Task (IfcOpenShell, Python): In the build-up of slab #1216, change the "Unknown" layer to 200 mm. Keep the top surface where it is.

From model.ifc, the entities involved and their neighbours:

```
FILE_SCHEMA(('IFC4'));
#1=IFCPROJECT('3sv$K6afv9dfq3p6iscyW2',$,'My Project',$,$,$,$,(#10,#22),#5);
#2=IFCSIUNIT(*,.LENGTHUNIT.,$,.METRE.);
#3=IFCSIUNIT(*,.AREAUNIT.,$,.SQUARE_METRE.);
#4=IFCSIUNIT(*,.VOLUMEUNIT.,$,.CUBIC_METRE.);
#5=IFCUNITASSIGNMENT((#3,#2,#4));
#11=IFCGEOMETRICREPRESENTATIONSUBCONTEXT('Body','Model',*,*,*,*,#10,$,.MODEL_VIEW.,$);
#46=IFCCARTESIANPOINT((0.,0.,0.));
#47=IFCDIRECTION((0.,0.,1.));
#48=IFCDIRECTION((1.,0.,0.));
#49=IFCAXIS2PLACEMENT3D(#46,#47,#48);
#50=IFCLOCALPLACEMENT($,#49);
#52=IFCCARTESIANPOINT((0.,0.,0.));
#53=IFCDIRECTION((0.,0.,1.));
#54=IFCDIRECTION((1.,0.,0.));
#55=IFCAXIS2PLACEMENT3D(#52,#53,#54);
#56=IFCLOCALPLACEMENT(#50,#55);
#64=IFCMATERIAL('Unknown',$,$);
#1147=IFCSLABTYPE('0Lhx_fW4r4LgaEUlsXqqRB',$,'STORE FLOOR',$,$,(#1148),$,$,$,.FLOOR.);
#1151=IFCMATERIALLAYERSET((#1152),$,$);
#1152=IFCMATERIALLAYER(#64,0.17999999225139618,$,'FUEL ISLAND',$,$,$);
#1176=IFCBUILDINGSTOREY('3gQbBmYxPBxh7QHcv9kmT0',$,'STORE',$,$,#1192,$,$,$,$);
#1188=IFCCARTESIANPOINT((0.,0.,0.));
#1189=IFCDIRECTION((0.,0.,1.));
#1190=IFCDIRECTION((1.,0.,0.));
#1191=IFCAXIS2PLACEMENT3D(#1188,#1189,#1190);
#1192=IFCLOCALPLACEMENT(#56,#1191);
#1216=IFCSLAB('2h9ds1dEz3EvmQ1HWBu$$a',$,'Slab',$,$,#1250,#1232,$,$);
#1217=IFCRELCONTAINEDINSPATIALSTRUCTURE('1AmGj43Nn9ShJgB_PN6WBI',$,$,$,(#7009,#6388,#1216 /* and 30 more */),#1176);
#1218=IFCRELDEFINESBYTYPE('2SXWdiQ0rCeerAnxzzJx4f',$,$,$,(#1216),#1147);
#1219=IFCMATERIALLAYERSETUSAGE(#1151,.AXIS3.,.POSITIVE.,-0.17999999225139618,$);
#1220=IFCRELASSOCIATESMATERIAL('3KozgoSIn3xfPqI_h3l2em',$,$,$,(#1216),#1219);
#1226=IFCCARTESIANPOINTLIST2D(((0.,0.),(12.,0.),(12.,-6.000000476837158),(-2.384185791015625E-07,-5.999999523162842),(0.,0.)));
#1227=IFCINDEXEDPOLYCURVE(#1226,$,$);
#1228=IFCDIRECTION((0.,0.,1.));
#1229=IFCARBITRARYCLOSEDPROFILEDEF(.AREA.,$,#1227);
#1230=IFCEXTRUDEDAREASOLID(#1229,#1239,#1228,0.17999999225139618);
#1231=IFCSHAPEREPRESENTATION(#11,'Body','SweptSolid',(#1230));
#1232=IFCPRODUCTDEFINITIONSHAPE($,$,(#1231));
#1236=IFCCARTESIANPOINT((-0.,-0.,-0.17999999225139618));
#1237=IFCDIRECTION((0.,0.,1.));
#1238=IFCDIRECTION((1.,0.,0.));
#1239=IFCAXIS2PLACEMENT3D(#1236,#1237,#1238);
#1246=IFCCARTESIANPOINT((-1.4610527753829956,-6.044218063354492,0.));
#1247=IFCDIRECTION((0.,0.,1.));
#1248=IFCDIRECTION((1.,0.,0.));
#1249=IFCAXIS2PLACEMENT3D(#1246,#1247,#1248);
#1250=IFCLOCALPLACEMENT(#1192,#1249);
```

```python
import ifcopenshell
import ifcopenshell.util.element
import ifcopenshell.util.representation
import ifcopenshell.util.unit

model = ifcopenshell.open("model.ifc")
unit_scale = ifcopenshell.util.unit.calculate_unit_scale(model)

layer_set = model.by_id(1151)
layer = next(l for l in layer_set.MaterialLayers if l.Material and l.Material.Name == "Unknown")
change = 0.2 / unit_scale - layer.LayerThickness
layer.LayerThickness += change

# Geometry does not follow the layer set by itself.
slabs = [e for e in ifcopenshell.util.element.get_elements_by_material(model, layer_set) if e.is_a("IfcSlab")]
for slab in sorted(slabs, key=lambda e: e.id()):
    body = ifcopenshell.util.representation.get_representation(slab, "Model", "Body")
    solid = body.Items[0]
    old_depth = solid.Depth
    solid.Depth += change
    # Extruded upwards: lower the start of the extrusion so the top stays.
    x, y, z = solid.Position.Location.Coordinates
    solid.Position.Location = model.createIfcCartesianPoint((x, y, z - change))
    print(slab.id(), f"{old_depth:g} -> {solid.Depth:g}")

# The layers are counted up from the underside, which has moved.
for usage in {ifcopenshell.util.element.get_material(slab) for slab in slabs}:
    usage.OffsetFromReferenceLine -= change

model.write("model_edited.ifc")
```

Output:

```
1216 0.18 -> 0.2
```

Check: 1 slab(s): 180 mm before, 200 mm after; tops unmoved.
